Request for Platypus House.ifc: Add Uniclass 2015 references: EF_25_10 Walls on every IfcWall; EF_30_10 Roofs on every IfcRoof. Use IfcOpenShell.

First a look at what the model holds.

```python
import ifcopenshell

model = ifcopenshell.open("Platypus House.ifc")
print(model.schema)
print("classifications:", [c.Name for c in model.by_type("IfcClassification")])
for ifc_class in ("IfcDoor", "IfcRoof", "IfcStair", "IfcWall", "IfcWindow"):
    print(ifc_class, len(model.by_type(ifc_class)))
```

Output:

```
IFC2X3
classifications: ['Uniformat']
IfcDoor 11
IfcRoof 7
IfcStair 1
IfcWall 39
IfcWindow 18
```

```python
import ifcopenshell
import ifcopenshell.api.classification

model = ifcopenshell.open("Platypus House.ifc")

# IFC2X3 requires Source and Edition and has no link from the project to the system.
system = model.create_entity("IfcClassification", Source="NBS", Edition="2015", Name="Uniclass 2015")

codes = {
    "IfcWall": ("EF_25_10", "Walls"),
    "IfcRoof": ("EF_30_10", "Roofs"),
}
for ifc_class, (code, name) in codes.items():
    products = model.by_type(ifc_class)
    ifcopenshell.api.classification.add_reference(
        model, products=products, classification=system, identification=code, name=name
    )
    print(code, len(products))

model.write("Platypus House_rev.ifc")
```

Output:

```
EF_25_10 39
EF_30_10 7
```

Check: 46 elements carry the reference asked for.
